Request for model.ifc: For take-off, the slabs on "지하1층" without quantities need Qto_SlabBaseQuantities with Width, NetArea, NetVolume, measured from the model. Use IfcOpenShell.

First a look at what the model holds.

```python
import ifcopenshell
import ifcopenshell.util.element
import ifcopenshell.util.unit

model = ifcopenshell.open("model.ifc")
print(model.schema)
for unit_type in ("LENGTHUNIT", "AREAUNIT", "VOLUMEUNIT"):
    print(unit_type, ifcopenshell.util.unit.calculate_unit_scale(model, unit_type))
storey = next(s for s in model.by_type("IfcBuildingStorey") if s.Name == "지하1층")
slabs = [e for e in ifcopenshell.util.element.get_decomposition(storey) if e.is_a("IfcSlab")]
for e in sorted(slabs, key=lambda e: e.id()):
    print(e.id(), e.is_a(), e.Name, list(ifcopenshell.util.element.get_psets(e, qtos_only=True)), sep=" | ")
```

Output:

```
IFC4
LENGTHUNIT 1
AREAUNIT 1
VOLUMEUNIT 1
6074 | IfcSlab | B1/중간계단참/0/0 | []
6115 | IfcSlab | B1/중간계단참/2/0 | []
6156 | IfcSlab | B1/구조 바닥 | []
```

```python
import ifcopenshell
import ifcopenshell.api.pset
import ifcopenshell.geom
import ifcopenshell.util.element
import ifcopenshell.util.shape
import ifcopenshell.util.unit

model = ifcopenshell.open("model.ifc")
unit_scale = ifcopenshell.util.unit.calculate_unit_scale(model)
area_scale = ifcopenshell.util.unit.calculate_unit_scale(model, "AREAUNIT")
volume_scale = ifcopenshell.util.unit.calculate_unit_scale(model, "VOLUMEUNIT")
settings = ifcopenshell.geom.settings()

storey = next(s for s in model.by_type("IfcBuildingStorey") if s.Name == "지하1층")
slabs = [e for e in ifcopenshell.util.element.get_decomposition(storey) if e.is_a("IfcSlab")]

for e in sorted(slabs, key=lambda e: e.id()):
    if ifcopenshell.util.element.get_psets(e, qtos_only=True, should_inherit=False):
        continue
    # Geometry comes back in metres, in the element's own axes.
    shape = ifcopenshell.geom.create_shape(settings, e)
    values = {
        "Width": ifcopenshell.util.shape.get_z(shape.geometry) / unit_scale,
        "NetArea": ifcopenshell.util.shape.get_footprint_area(shape.geometry) / area_scale,
        "NetVolume": ifcopenshell.util.shape.get_volume(shape.geometry) / volume_scale,
    }
    qto = ifcopenshell.api.pset.add_qto(model, product=e, name="Qto_SlabBaseQuantities")
    ifcopenshell.api.pset.edit_qto(model, qto=qto, properties=values)
    print(e.id(), {k: round(v, 3) for k, v in values.items()})

model.write("model_v2.ifc")
```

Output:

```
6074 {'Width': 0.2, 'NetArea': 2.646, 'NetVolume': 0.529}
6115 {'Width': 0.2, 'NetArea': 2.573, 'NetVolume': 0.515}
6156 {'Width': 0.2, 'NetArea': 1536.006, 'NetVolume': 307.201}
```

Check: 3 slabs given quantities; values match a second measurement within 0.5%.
